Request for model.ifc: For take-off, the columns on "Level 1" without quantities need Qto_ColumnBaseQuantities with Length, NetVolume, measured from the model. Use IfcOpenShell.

First a look at what the model holds.

```python
import ifcopenshell
import ifcopenshell.util.element
import ifcopenshell.util.unit

model = ifcopenshell.open("model.ifc")
print(model.schema)
for unit_type in ("LENGTHUNIT", "AREAUNIT", "VOLUMEUNIT"):
    print(unit_type, ifcopenshell.util.unit.calculate_unit_scale(model, unit_type))
storey = next(s for s in model.by_type("IfcBuildingStorey") if s.Name == "Level 1")
columns = [e for e in ifcopenshell.util.element.get_decomposition(storey) if e.is_a("IfcColumn")]
for e in sorted(columns, key=lambda e: e.id()):
    print(e.id(), e.is_a(), e.Name, list(ifcopenshell.util.element.get_psets(e, qtos_only=True)), sep=" | ")
```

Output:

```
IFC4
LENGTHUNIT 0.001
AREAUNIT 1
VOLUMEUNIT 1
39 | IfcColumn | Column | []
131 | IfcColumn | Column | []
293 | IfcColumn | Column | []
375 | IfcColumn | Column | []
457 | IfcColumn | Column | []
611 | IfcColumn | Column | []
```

```python
import ifcopenshell
import ifcopenshell.api.pset
import ifcopenshell.geom
import ifcopenshell.util.element
import ifcopenshell.util.shape
import ifcopenshell.util.unit

model = ifcopenshell.open("model.ifc")
unit_scale = ifcopenshell.util.unit.calculate_unit_scale(model)
volume_scale = ifcopenshell.util.unit.calculate_unit_scale(model, "VOLUMEUNIT")
settings = ifcopenshell.geom.settings()

storey = next(s for s in model.by_type("IfcBuildingStorey") if s.Name == "Level 1")
columns = [e for e in ifcopenshell.util.element.get_decomposition(storey) if e.is_a("IfcColumn")]

for e in sorted(columns, key=lambda e: e.id()):
    if ifcopenshell.util.element.get_psets(e, qtos_only=True, should_inherit=False):
        continue
    # Geometry comes back in metres, in the element's own axes.
    shape = ifcopenshell.geom.create_shape(settings, e)
    values = {
        "Length": ifcopenshell.util.shape.get_z(shape.geometry) / unit_scale,
        "NetVolume": ifcopenshell.util.shape.get_volume(shape.geometry) / volume_scale,
    }
    qto = ifcopenshell.api.pset.add_qto(model, product=e, name="Qto_ColumnBaseQuantities")
    ifcopenshell.api.pset.edit_qto(model, qto=qto, properties=values)
    print(e.id(), {k: round(v, 3) for k, v in values.items()})

model.write("model_rev.ifc")
```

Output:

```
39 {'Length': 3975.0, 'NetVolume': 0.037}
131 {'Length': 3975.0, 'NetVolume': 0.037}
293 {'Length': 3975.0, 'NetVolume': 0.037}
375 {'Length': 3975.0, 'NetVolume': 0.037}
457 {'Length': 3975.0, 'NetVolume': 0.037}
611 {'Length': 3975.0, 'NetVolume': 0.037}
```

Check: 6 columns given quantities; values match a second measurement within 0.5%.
